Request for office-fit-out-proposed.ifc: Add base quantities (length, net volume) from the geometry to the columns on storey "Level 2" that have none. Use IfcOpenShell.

First a look at what the model holds.

```python
import ifcopenshell
import ifcopenshell.util.element
import ifcopenshell.util.unit

model = ifcopenshell.open("office-fit-out-proposed.ifc")
print(model.schema)
for unit_type in ("LENGTHUNIT", "AREAUNIT", "VOLUMEUNIT"):
    print(unit_type, ifcopenshell.util.unit.calculate_unit_scale(model, unit_type))
storey = next(s for s in model.by_type("IfcBuildingStorey") if s.Name == "Level 2")
columns = [e for e in ifcopenshell.util.element.get_decomposition(storey) if e.is_a("IfcColumn")]
for e in sorted(columns, key=lambda e: e.id()):
    print(e.id(), e.is_a(), e.Name, list(ifcopenshell.util.element.get_psets(e, qtos_only=True)), sep=" | ")
```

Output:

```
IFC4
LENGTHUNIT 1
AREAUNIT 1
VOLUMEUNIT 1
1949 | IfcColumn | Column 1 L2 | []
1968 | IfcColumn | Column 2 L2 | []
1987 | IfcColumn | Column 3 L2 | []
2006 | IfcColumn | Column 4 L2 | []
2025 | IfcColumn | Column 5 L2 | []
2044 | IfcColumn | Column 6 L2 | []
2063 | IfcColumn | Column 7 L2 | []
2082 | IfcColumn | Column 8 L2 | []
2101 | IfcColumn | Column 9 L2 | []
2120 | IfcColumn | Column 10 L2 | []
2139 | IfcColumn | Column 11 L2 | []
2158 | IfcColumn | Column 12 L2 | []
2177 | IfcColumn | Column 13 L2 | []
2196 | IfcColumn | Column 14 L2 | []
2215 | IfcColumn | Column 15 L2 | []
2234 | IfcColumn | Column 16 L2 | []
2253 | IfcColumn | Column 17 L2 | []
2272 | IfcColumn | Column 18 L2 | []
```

```python
import ifcopenshell
import ifcopenshell.api.pset
import ifcopenshell.geom
import ifcopenshell.util.element
import ifcopenshell.util.shape
import ifcopenshell.util.unit

model = ifcopenshell.open("office-fit-out-proposed.ifc")
unit_scale = ifcopenshell.util.unit.calculate_unit_scale(model)
volume_scale = ifcopenshell.util.unit.calculate_unit_scale(model, "VOLUMEUNIT")
settings = ifcopenshell.geom.settings()

storey = next(s for s in model.by_type("IfcBuildingStorey") if s.Name == "Level 2")
columns = [e for e in ifcopenshell.util.element.get_decomposition(storey) if e.is_a("IfcColumn")]

for e in sorted(columns, key=lambda e: e.id()):
    if ifcopenshell.util.element.get_psets(e, qtos_only=True, should_inherit=False):
        continue
    # Geometry comes back in metres, in the element's own axes.
    shape = ifcopenshell.geom.create_shape(settings, e)
    values = {
        "Length": ifcopenshell.util.shape.get_z(shape.geometry) / unit_scale,
        "NetVolume": ifcopenshell.util.shape.get_volume(shape.geometry) / volume_scale,
    }
    qto = ifcopenshell.api.pset.add_qto(model, product=e, name="Qto_ColumnBaseQuantities")
    ifcopenshell.api.pset.edit_qto(model, qto=qto, properties=values)
    print(e.id(), {k: round(v, 3) for k, v in values.items()})

model.write("office-fit-out-proposed_edited.ifc")
```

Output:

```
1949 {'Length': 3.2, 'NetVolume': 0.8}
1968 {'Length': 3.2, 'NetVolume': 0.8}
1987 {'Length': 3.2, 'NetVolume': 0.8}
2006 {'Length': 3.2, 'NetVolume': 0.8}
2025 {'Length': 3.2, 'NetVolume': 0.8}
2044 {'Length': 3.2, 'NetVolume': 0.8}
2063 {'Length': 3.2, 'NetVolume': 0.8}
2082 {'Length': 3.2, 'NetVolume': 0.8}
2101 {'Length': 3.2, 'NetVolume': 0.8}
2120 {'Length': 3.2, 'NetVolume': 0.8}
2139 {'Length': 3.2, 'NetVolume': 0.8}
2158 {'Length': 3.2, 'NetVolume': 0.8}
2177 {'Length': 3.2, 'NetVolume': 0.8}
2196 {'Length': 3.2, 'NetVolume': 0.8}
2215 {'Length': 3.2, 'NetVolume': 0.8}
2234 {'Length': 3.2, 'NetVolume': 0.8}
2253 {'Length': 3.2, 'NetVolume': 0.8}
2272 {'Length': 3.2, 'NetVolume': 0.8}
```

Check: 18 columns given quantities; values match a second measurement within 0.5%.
